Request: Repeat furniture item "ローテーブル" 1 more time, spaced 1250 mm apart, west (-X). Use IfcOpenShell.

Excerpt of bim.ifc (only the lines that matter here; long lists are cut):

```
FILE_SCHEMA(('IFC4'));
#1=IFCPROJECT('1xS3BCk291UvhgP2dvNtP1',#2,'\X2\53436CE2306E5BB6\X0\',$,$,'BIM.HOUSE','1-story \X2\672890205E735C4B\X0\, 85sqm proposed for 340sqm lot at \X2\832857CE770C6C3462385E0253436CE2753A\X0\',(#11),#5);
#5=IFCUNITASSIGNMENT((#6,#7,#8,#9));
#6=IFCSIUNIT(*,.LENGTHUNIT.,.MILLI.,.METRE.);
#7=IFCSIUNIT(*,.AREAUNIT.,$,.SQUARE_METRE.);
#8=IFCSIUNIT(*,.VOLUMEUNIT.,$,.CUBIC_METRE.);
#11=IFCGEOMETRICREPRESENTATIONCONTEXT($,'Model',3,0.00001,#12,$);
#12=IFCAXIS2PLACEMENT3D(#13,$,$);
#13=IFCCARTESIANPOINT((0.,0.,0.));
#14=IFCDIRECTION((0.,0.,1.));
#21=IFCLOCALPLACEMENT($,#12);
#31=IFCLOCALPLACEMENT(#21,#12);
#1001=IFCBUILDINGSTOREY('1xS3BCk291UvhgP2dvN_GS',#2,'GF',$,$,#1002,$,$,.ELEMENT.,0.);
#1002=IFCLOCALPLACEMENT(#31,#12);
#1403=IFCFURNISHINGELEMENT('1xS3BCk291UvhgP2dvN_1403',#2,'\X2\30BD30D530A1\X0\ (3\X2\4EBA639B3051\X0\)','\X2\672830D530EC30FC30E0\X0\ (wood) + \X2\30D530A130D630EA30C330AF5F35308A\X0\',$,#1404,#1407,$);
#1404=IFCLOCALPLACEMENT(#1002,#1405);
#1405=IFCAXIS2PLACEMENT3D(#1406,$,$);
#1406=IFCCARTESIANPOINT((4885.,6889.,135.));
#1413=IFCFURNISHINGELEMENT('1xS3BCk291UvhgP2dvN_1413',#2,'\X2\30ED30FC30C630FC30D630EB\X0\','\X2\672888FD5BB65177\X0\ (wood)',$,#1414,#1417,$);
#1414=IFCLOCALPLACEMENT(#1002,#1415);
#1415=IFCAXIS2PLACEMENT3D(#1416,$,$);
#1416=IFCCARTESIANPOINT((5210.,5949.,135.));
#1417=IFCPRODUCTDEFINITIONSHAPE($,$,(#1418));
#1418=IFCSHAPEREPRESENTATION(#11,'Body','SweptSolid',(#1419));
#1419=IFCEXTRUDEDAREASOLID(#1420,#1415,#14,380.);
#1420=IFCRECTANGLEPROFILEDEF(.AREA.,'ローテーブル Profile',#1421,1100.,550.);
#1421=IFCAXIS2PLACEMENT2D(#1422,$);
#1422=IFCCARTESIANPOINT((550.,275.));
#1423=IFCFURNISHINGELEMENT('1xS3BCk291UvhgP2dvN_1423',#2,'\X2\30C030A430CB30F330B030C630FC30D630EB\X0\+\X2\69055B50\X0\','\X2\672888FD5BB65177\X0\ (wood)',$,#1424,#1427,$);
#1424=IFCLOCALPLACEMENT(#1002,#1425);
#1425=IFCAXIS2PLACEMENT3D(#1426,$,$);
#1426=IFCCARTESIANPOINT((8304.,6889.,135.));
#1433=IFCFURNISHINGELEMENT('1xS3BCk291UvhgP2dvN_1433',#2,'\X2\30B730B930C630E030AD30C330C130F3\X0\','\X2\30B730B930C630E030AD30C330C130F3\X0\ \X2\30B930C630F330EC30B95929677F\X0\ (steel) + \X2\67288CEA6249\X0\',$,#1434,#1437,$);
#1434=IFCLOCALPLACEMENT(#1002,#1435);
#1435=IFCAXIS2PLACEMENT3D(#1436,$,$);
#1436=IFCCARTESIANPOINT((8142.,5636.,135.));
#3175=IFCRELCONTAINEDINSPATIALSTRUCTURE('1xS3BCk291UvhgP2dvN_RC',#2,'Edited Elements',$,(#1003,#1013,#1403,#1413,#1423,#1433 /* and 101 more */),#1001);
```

```python
import numpy as np
import ifcopenshell
import ifcopenshell.api.geometry
import ifcopenshell.api.root
import ifcopenshell.util.element
import ifcopenshell.util.placement

model = ifcopenshell.open("bim.ifc")


def reuse_history(source, copy):
    """copy_class also copies each property set's owner history, people and application; keep the originals."""
    for rel in copy.IsDefinedBy:
        if rel.is_a("IfcRelDefinesByProperties") and (history := rel.RelatingPropertyDefinition.OwnerHistory):
            rel.RelatingPropertyDefinition.OwnerHistory = source.OwnerHistory
            ifcopenshell.util.element.remove_deep2(model, history)


source = model.by_guid("1xS3BCk291UvhgP2dvN_1413")
base = ifcopenshell.util.placement.get_local_placement(source.ObjectPlacement)
step = np.array([-1.0, 0.0, 0.0]) * 1250.0

for i in range(1, 2):
    copy = ifcopenshell.api.root.copy_class(model, product=source)
    copy.Representation = ifcopenshell.util.element.copy_deep(
        model, source.Representation, exclude=["IfcGeometricRepresentationContext", "IfcRepresentationMap"]
    )
    reuse_history(source, copy)
    matrix = base.copy()
    matrix[:3, 3] += i * step
    print("added at", matrix[:3, 3].round(3) + 0.0)
    ifcopenshell.api.geometry.edit_object_placement(model, product=copy, matrix=matrix, is_si=False)

model.write("bim-out.ifc")
```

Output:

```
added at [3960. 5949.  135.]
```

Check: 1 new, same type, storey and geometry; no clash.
